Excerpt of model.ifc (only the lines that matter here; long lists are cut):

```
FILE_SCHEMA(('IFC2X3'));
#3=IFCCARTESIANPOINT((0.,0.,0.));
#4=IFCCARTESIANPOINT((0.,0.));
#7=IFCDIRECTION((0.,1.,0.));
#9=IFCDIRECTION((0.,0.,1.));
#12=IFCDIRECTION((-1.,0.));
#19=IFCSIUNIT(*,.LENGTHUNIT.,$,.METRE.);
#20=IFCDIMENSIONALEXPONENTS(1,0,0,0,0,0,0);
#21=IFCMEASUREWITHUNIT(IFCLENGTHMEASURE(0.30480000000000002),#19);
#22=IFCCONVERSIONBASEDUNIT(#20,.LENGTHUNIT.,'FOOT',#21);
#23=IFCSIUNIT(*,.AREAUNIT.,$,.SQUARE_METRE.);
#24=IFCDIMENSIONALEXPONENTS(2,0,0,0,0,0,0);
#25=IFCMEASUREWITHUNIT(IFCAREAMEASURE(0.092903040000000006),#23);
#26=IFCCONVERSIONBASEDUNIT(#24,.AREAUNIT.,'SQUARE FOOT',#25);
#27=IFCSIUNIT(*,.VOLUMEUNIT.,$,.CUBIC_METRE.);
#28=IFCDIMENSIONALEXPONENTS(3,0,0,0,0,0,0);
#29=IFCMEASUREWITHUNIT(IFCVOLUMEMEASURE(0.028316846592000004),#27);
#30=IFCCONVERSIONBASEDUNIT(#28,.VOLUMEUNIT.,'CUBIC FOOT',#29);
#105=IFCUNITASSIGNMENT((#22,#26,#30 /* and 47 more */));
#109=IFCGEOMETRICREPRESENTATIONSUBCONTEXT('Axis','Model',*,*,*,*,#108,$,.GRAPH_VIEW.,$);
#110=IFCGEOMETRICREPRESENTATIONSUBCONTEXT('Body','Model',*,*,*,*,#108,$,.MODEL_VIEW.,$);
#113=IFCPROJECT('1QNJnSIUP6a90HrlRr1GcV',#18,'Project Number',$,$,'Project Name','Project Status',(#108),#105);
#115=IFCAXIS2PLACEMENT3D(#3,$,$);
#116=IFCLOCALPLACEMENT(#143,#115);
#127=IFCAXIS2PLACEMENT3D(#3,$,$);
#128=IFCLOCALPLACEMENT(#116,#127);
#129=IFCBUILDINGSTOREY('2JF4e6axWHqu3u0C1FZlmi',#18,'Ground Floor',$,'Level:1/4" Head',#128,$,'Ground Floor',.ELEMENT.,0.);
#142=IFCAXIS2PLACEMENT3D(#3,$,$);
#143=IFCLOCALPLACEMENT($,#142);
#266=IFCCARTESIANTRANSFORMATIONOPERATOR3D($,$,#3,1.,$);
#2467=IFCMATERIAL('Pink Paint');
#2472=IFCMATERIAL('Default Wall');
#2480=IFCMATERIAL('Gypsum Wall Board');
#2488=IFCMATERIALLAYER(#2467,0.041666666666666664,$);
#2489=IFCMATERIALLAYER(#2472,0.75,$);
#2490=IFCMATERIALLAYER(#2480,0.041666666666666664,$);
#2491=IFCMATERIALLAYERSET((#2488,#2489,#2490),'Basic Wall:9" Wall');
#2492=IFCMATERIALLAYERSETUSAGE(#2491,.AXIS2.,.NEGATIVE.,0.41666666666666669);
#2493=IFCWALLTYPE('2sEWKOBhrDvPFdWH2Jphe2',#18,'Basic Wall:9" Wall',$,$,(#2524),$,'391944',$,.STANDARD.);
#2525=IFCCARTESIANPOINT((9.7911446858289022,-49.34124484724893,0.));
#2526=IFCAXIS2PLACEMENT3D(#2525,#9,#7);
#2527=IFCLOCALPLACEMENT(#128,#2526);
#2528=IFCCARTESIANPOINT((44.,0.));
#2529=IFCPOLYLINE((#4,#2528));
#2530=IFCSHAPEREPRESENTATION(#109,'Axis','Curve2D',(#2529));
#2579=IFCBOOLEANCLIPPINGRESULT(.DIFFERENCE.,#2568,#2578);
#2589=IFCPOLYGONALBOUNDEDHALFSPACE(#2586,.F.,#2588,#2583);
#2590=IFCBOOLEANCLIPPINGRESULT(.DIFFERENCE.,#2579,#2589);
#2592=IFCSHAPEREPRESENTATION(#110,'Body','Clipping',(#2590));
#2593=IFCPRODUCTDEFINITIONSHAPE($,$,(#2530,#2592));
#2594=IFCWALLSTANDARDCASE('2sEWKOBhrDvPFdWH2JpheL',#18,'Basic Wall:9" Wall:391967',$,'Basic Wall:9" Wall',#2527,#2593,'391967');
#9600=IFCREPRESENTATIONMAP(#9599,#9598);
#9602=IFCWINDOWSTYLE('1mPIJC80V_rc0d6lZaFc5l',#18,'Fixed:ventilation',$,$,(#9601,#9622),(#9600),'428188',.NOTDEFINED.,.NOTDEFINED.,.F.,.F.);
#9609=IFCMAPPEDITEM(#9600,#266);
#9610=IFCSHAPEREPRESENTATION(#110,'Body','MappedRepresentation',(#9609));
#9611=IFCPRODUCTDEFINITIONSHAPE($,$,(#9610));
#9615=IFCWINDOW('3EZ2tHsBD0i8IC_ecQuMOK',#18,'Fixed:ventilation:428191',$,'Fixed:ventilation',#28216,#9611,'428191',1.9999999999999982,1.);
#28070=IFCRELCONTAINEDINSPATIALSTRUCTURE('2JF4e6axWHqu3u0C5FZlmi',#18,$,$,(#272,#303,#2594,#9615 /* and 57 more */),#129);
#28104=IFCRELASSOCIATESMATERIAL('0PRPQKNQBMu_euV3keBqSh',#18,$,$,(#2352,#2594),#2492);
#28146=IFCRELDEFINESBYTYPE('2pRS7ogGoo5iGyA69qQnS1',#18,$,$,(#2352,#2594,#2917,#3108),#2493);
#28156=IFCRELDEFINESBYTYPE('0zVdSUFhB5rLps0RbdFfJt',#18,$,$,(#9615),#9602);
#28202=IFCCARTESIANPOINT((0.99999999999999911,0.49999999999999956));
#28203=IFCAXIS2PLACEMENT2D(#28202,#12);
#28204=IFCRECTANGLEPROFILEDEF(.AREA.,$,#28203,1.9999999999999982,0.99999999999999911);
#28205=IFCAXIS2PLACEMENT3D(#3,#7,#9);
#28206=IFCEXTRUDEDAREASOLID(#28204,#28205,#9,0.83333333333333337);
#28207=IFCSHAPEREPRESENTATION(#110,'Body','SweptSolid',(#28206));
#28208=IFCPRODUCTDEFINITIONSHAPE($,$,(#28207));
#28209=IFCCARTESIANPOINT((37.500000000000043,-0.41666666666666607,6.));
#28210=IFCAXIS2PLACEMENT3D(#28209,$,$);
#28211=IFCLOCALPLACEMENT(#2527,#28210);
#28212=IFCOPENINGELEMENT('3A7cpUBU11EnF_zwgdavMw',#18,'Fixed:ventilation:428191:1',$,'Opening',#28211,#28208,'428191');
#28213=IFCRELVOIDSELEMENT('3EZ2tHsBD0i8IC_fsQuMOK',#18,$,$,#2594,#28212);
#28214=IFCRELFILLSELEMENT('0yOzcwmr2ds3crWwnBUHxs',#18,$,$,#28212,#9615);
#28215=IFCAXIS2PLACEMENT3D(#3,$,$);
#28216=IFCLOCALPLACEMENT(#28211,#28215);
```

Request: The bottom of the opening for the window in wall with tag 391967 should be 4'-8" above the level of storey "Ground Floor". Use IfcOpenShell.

```python
import numpy as np
import ifcopenshell
import ifcopenshell.api.geometry
import ifcopenshell.geom
import ifcopenshell.util.element
import ifcopenshell.util.placement
import ifcopenshell.util.shape
import ifcopenshell.util.unit

model = ifcopenshell.open("model.ifc")
unit_scale = ifcopenshell.util.unit.calculate_unit_scale(model)

window = model.by_guid("3EZ2tHsBD0i8IC_ecQuMOK")
opening = window.FillsVoids[0].RelatingOpeningElement
storey = ifcopenshell.util.element.get_container(window, ifc_class="IfcBuildingStorey")
level = ifcopenshell.util.placement.get_local_placement(storey.ObjectPlacement)[2, 3]

# The opening's origin need not be at the sill, so measure its lowest point.
shape = ifcopenshell.geom.create_shape(ifcopenshell.geom.settings(), opening)
bottom = ifcopenshell.util.shape.get_shape_bottom_elevation(shape, shape.geometry) / unit_scale
dz = level + 56 * 0.0254 / unit_scale - bottom

shift = np.array([0.0, 0.0, dz])
# The window is placed relative to its opening, so it follows when the opening moves.
matrix = ifcopenshell.util.placement.get_local_placement(opening.ObjectPlacement)
matrix[:3, 3] += shift
ifcopenshell.api.geometry.edit_object_placement(
    model, product=opening, matrix=matrix, is_si=False, should_transform_children=True
)

print(f"moved by {dz * unit_scale:+.3f} m")

model.write("model_edited.ifc")
```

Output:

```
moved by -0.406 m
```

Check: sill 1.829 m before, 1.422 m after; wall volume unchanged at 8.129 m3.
